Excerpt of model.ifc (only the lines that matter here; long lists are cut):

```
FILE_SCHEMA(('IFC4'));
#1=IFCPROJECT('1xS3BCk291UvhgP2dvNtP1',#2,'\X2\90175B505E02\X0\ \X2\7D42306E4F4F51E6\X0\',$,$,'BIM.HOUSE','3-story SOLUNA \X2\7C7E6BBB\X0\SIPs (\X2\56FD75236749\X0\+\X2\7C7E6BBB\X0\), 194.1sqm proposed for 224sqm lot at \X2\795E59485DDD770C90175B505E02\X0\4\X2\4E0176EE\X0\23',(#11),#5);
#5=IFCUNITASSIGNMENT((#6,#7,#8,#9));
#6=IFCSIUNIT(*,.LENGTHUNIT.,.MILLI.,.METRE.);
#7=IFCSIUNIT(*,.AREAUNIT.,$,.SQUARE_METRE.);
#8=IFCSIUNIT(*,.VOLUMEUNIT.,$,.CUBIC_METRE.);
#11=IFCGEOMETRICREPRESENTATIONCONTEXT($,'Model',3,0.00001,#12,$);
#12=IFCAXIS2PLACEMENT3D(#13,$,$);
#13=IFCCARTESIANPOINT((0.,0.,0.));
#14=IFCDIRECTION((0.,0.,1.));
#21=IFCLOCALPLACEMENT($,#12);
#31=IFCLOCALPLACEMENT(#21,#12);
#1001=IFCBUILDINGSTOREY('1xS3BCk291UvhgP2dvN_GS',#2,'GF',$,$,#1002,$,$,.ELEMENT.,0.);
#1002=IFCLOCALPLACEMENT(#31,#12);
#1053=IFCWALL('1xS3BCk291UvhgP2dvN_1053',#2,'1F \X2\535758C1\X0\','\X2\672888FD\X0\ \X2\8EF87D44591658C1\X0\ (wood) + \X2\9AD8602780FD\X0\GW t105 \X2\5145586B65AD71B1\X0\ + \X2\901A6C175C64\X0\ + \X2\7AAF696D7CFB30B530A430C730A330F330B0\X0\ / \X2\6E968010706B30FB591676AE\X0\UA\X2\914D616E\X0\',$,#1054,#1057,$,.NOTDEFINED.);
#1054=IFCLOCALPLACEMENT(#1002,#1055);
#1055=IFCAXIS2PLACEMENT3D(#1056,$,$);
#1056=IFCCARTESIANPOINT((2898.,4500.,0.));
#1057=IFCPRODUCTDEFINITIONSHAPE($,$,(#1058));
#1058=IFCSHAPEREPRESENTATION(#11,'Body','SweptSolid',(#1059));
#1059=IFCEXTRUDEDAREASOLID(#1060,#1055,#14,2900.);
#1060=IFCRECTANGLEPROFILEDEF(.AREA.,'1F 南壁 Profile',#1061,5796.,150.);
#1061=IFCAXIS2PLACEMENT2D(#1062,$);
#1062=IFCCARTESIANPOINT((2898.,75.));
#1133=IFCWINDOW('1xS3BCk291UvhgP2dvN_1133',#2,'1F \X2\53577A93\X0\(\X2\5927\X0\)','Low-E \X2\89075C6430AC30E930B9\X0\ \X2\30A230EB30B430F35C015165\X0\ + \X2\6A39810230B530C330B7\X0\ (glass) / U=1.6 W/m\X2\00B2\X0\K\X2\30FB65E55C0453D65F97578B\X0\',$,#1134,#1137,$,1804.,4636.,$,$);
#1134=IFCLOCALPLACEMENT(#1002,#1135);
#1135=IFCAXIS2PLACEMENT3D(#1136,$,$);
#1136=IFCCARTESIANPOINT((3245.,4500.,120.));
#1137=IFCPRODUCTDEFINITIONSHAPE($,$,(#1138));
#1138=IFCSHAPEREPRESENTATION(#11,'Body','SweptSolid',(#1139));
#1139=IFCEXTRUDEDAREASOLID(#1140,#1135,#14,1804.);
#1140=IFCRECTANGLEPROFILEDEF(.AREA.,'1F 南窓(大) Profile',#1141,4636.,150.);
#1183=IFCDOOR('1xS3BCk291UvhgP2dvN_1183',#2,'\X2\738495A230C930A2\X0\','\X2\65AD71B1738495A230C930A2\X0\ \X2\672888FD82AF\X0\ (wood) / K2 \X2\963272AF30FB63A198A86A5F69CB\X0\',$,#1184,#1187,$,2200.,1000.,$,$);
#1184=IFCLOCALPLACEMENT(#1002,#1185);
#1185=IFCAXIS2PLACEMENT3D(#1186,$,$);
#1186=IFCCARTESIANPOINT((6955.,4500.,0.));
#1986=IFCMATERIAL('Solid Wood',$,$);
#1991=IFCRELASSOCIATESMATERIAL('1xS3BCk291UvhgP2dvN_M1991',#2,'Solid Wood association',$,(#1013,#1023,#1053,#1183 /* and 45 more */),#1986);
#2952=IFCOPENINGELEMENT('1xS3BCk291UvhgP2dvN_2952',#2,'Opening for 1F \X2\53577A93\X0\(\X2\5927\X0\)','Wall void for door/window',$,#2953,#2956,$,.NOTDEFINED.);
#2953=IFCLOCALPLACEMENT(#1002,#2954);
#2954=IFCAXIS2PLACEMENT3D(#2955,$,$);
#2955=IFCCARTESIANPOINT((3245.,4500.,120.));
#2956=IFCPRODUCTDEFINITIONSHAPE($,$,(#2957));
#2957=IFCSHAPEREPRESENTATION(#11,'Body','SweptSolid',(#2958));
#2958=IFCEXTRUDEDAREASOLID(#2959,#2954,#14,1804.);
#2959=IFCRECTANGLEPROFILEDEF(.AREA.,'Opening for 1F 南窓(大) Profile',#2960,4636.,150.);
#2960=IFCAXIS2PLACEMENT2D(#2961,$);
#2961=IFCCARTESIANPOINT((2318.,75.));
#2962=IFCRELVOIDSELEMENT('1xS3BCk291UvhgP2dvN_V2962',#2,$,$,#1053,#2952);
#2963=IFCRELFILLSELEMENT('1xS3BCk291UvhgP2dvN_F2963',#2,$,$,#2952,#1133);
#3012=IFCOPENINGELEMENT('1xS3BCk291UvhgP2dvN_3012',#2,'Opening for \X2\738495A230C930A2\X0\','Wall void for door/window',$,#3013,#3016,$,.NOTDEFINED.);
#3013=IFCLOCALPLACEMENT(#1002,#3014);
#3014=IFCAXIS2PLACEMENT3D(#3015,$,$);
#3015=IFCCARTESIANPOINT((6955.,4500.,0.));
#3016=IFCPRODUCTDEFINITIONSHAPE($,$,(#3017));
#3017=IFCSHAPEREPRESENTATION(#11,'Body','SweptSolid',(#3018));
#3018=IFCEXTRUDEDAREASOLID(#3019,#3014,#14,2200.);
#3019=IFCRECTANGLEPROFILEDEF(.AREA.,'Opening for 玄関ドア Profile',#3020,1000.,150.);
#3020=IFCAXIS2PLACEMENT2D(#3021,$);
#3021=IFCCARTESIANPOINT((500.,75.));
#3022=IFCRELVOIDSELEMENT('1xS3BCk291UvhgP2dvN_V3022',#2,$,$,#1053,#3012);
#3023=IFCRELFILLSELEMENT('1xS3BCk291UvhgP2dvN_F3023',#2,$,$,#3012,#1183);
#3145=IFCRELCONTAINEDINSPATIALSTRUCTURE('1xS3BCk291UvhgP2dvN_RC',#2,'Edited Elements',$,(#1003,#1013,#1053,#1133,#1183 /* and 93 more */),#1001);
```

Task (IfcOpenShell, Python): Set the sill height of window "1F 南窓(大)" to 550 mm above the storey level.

```python
import numpy as np
import ifcopenshell
import ifcopenshell.api.geometry
import ifcopenshell.geom
import ifcopenshell.util.element
import ifcopenshell.util.placement
import ifcopenshell.util.shape
import ifcopenshell.util.unit

model = ifcopenshell.open("model.ifc")
unit_scale = ifcopenshell.util.unit.calculate_unit_scale(model)

window = model.by_id(1133)
opening = window.FillsVoids[0].RelatingOpeningElement
storey = ifcopenshell.util.element.get_container(window, ifc_class="IfcBuildingStorey")
level = ifcopenshell.util.placement.get_local_placement(storey.ObjectPlacement)[2, 3]

# The opening's origin need not be at the sill, so measure its lowest point.
shape = ifcopenshell.geom.create_shape(ifcopenshell.geom.settings(), opening)
bottom = ifcopenshell.util.shape.get_shape_bottom_elevation(shape, shape.geometry) / unit_scale
dz = level + 0.55 / unit_scale - bottom

shift = np.array([0.0, 0.0, dz])
# The window is not placed relative to its opening, so move both.
for product in (opening, window):
    matrix = ifcopenshell.util.placement.get_local_placement(product.ObjectPlacement)
    matrix[:3, 3] += shift
    ifcopenshell.api.geometry.edit_object_placement(model, product=product, matrix=matrix, is_si=False)

print(f"moved by {dz * unit_scale:+.3f} m")

model.write("model_v2.ifc")
```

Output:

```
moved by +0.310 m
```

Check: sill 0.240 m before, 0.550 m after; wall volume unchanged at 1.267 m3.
